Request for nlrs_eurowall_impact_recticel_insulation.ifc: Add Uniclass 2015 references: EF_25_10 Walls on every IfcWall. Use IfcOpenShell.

First a look at what the model holds.

```python
import ifcopenshell

model = ifcopenshell.open("nlrs_eurowall_impact_recticel_insulation.ifc")
print(model.schema)
print("classifications:", [c.Name for c in model.by_type("IfcClassification")])
for ifc_class in ("IfcDoor", "IfcRoof", "IfcStair", "IfcWall", "IfcWindow"):
    print(ifc_class, len(model.by_type(ifc_class)))
```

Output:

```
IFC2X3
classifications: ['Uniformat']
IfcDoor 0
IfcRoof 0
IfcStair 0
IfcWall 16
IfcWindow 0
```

```python
import ifcopenshell
import ifcopenshell.api.classification

model = ifcopenshell.open("nlrs_eurowall_impact_recticel_insulation.ifc")

# IFC2X3 requires Source and Edition and has no link from the project to the system.
system = model.create_entity("IfcClassification", Source="NBS", Edition="2015", Name="Uniclass 2015")

codes = {
    "IfcWall": ("EF_25_10", "Walls"),
}
for ifc_class, (code, name) in codes.items():
    products = model.by_type(ifc_class)
    ifcopenshell.api.classification.add_reference(
        model, products=products, classification=system, identification=code, name=name
    )
    print(code, len(products))

model.write("nlrs_eurowall_impact_recticel_insulation_v2.ifc")
```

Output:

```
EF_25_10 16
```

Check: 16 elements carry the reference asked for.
